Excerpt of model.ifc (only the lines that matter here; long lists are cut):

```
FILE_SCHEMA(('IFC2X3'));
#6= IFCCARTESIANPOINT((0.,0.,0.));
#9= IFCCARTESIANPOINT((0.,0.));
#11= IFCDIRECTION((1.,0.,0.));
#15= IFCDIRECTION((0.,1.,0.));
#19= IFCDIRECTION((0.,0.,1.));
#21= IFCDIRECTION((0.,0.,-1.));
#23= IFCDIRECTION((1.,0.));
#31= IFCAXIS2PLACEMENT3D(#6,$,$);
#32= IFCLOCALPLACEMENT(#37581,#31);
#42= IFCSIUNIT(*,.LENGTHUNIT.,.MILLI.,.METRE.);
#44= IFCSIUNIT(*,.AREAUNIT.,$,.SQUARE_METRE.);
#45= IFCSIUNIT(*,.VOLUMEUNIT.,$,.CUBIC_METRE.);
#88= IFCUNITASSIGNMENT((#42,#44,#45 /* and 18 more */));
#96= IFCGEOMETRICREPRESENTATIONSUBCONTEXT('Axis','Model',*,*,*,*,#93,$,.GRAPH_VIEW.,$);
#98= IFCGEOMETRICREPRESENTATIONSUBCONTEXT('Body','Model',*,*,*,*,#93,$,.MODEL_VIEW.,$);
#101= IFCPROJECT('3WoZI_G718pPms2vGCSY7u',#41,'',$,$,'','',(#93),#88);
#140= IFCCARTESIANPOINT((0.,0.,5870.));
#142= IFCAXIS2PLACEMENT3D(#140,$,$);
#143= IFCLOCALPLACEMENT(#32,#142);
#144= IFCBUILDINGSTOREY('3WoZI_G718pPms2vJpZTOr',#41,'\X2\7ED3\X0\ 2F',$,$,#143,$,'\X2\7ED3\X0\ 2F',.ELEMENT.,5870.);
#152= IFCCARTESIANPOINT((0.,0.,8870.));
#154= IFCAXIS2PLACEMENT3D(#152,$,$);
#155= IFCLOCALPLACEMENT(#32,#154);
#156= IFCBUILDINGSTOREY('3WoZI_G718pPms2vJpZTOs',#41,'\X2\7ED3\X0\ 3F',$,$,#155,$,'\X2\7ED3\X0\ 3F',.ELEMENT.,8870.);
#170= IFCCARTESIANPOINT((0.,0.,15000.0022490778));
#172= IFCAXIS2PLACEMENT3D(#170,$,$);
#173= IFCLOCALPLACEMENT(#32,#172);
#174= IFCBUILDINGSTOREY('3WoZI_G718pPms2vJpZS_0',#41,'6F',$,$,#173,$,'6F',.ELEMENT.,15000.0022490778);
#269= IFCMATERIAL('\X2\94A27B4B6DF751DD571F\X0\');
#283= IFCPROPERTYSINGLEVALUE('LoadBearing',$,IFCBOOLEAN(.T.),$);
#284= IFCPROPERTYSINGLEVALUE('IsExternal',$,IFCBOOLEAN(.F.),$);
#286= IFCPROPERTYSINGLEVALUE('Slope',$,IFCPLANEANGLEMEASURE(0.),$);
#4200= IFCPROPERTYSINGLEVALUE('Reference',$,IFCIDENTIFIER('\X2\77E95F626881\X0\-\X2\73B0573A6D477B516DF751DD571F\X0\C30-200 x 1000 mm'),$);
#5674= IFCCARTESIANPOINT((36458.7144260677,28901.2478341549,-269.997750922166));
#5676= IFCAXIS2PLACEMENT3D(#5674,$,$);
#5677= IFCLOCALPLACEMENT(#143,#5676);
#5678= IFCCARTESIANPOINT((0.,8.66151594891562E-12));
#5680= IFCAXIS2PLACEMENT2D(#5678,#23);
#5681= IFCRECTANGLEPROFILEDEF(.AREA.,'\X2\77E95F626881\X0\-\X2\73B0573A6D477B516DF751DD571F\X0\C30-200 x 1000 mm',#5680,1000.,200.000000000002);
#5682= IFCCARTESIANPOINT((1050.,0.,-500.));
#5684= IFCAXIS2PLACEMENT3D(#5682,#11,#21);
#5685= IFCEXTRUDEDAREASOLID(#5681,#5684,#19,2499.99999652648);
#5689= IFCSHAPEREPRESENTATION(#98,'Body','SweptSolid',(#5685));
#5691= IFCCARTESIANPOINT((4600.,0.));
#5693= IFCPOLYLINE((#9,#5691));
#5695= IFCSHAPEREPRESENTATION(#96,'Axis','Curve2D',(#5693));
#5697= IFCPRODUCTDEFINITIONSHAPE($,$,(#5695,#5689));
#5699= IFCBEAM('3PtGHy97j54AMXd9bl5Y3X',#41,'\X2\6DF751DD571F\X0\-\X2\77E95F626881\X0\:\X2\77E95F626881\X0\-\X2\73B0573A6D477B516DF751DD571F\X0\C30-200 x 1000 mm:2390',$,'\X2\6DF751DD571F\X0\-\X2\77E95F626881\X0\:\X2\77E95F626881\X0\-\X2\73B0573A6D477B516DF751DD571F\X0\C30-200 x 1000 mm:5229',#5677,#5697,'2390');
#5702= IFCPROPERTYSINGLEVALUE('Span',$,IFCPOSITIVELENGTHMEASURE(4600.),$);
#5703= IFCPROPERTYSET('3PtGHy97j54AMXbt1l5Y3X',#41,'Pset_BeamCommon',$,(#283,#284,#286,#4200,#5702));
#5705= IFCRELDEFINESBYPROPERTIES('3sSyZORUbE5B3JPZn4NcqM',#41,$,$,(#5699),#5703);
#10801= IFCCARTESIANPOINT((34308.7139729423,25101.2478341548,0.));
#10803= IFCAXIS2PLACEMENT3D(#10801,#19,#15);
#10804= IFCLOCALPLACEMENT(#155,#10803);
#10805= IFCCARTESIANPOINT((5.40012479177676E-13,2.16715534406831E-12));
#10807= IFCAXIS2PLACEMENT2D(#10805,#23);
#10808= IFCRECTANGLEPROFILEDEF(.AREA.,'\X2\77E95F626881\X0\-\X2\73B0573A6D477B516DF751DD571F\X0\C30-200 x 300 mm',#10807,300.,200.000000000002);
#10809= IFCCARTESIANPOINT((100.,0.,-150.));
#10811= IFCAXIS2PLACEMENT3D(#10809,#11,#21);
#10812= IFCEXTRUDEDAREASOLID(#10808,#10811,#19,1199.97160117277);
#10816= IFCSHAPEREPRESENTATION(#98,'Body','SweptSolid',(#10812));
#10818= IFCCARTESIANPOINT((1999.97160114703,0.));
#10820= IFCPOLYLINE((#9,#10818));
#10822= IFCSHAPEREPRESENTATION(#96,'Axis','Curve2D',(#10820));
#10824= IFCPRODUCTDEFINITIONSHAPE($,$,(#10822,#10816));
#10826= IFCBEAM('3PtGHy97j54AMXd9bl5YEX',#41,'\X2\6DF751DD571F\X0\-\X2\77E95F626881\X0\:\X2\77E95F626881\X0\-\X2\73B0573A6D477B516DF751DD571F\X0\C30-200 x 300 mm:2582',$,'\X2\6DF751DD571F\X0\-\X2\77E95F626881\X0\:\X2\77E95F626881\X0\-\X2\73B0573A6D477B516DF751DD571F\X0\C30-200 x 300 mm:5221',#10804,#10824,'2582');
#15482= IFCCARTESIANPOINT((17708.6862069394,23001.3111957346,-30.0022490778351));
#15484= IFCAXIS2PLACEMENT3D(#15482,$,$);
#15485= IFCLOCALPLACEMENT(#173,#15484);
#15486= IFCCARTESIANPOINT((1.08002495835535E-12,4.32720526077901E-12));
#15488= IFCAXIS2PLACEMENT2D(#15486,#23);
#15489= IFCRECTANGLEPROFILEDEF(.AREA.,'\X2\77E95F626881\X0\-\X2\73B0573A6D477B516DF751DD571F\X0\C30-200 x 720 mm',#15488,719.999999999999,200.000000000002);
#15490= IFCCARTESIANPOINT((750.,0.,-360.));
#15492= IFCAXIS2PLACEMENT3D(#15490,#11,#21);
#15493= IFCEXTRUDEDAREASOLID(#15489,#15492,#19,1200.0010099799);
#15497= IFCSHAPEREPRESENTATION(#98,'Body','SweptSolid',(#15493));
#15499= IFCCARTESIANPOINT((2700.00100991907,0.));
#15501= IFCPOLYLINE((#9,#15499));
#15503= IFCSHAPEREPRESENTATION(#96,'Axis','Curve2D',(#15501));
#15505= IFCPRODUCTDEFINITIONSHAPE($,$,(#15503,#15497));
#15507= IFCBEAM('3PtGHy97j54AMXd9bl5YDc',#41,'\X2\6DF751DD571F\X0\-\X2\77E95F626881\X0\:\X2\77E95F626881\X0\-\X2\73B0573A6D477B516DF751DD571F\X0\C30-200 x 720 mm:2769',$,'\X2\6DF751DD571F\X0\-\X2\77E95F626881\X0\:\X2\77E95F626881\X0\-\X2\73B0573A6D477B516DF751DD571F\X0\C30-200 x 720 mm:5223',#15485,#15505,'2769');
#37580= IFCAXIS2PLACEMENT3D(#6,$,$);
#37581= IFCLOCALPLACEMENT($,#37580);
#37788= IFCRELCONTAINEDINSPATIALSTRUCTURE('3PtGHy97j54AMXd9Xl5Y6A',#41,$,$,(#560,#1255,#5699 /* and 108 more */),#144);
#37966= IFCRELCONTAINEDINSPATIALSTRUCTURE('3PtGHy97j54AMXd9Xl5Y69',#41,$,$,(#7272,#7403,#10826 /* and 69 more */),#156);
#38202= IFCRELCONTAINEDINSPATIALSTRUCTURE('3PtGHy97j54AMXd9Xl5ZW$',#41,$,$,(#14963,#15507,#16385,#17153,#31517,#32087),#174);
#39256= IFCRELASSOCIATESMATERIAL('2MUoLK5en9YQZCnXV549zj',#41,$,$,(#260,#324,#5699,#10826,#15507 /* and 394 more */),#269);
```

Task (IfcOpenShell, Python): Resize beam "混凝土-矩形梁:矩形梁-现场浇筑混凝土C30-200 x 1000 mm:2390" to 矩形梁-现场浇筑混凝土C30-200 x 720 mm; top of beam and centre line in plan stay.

```python
import ifcopenshell
import ifcopenshell.api.pset
import ifcopenshell.util.element
import ifcopenshell.util.representation

model = ifcopenshell.open("model.ifc")

member = model.by_id(5699)
source = next(p for p in model.by_type("IfcRectangleProfileDef") if p.ProfileName == "矩形梁-现场浇筑混凝土C30-200 x 720 mm")

body = ifcopenshell.util.representation.get_representation(member, "Model", "Body")
solid = body.Items[0]
old_profile = solid.SweptArea

# Copy the section's sizes but keep this member's own profile position.
profile = ifcopenshell.util.element.copy(model, source)
# Profiles are centred, so shift by half the change in depth to hold the top.
shift = (old_profile.XDim - profile.XDim) / 2
x, y = old_profile.Position.Location.Coordinates
up = (-1.0, 0.0)  # upwards, in the solid's own plane
location = model.createIfcCartesianPoint((x + up[0] * shift, y + up[1] * shift))
profile.Position = model.createIfcAxis2Placement2D(location, old_profile.Position.RefDirection)
solid.SweptArea = profile
if not model.get_total_inverses(old_profile):
    ifcopenshell.util.element.remove_deep2(model, old_profile)
member.Name = member.Name.replace("矩形梁-现场浇筑混凝土C30-200 x 1000 mm", "矩形梁-现场浇筑混凝土C30-200 x 720 mm")
member.ObjectType = member.ObjectType.replace("矩形梁-现场浇筑混凝土C30-200 x 1000 mm", "矩形梁-现场浇筑混凝土C30-200 x 720 mm")
pset = model.by_id(ifcopenshell.util.element.get_pset(member, "Pset_BeamCommon", should_inherit=False)["id"])
ifcopenshell.api.pset.edit_pset(model, pset=pset, properties={"Reference": "矩形梁-现场浇筑混凝土C30-200 x 720 mm"})

print(solid.SweptArea)

model.write("model-out.ifc")
```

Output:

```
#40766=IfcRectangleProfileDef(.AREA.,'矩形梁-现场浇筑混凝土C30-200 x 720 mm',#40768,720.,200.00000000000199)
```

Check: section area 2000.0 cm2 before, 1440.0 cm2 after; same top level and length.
